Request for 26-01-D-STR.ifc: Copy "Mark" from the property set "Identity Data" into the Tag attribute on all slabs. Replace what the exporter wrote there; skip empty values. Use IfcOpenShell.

First a look at what the model holds.

```python
import ifcopenshell
import ifcopenshell.util.element

model = ifcopenshell.open("26-01-D-STR.ifc")
print(model.schema)
slabs = model.by_type("IfcSlab")
print(len(slabs), "slabs")
for e in slabs[:8]:
    source = ifcopenshell.util.element.get_pset(e, "Identity Data", "Mark")
    target = e.Tag
    print(e.id(), repr(source), repr(target), sep=" | ")
```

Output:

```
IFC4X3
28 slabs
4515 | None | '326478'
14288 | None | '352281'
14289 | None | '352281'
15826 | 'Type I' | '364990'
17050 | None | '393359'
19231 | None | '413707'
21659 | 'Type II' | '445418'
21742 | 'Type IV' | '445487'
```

```python
import ifcopenshell
import ifcopenshell.util.element

model = ifcopenshell.open("26-01-D-STR.ifc")

count = 0
for e in model.by_type("IfcSlab"):
    value = ifcopenshell.util.element.get_pset(e, "Identity Data", "Mark")
    current = e.Tag
    if not value or not value.strip() or current == value:
        continue
    e.Tag = value
    count += 1

print(count, "slabs updated")

model.write("26-01-D-STR_v2.ifc")
```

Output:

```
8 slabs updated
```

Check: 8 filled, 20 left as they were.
